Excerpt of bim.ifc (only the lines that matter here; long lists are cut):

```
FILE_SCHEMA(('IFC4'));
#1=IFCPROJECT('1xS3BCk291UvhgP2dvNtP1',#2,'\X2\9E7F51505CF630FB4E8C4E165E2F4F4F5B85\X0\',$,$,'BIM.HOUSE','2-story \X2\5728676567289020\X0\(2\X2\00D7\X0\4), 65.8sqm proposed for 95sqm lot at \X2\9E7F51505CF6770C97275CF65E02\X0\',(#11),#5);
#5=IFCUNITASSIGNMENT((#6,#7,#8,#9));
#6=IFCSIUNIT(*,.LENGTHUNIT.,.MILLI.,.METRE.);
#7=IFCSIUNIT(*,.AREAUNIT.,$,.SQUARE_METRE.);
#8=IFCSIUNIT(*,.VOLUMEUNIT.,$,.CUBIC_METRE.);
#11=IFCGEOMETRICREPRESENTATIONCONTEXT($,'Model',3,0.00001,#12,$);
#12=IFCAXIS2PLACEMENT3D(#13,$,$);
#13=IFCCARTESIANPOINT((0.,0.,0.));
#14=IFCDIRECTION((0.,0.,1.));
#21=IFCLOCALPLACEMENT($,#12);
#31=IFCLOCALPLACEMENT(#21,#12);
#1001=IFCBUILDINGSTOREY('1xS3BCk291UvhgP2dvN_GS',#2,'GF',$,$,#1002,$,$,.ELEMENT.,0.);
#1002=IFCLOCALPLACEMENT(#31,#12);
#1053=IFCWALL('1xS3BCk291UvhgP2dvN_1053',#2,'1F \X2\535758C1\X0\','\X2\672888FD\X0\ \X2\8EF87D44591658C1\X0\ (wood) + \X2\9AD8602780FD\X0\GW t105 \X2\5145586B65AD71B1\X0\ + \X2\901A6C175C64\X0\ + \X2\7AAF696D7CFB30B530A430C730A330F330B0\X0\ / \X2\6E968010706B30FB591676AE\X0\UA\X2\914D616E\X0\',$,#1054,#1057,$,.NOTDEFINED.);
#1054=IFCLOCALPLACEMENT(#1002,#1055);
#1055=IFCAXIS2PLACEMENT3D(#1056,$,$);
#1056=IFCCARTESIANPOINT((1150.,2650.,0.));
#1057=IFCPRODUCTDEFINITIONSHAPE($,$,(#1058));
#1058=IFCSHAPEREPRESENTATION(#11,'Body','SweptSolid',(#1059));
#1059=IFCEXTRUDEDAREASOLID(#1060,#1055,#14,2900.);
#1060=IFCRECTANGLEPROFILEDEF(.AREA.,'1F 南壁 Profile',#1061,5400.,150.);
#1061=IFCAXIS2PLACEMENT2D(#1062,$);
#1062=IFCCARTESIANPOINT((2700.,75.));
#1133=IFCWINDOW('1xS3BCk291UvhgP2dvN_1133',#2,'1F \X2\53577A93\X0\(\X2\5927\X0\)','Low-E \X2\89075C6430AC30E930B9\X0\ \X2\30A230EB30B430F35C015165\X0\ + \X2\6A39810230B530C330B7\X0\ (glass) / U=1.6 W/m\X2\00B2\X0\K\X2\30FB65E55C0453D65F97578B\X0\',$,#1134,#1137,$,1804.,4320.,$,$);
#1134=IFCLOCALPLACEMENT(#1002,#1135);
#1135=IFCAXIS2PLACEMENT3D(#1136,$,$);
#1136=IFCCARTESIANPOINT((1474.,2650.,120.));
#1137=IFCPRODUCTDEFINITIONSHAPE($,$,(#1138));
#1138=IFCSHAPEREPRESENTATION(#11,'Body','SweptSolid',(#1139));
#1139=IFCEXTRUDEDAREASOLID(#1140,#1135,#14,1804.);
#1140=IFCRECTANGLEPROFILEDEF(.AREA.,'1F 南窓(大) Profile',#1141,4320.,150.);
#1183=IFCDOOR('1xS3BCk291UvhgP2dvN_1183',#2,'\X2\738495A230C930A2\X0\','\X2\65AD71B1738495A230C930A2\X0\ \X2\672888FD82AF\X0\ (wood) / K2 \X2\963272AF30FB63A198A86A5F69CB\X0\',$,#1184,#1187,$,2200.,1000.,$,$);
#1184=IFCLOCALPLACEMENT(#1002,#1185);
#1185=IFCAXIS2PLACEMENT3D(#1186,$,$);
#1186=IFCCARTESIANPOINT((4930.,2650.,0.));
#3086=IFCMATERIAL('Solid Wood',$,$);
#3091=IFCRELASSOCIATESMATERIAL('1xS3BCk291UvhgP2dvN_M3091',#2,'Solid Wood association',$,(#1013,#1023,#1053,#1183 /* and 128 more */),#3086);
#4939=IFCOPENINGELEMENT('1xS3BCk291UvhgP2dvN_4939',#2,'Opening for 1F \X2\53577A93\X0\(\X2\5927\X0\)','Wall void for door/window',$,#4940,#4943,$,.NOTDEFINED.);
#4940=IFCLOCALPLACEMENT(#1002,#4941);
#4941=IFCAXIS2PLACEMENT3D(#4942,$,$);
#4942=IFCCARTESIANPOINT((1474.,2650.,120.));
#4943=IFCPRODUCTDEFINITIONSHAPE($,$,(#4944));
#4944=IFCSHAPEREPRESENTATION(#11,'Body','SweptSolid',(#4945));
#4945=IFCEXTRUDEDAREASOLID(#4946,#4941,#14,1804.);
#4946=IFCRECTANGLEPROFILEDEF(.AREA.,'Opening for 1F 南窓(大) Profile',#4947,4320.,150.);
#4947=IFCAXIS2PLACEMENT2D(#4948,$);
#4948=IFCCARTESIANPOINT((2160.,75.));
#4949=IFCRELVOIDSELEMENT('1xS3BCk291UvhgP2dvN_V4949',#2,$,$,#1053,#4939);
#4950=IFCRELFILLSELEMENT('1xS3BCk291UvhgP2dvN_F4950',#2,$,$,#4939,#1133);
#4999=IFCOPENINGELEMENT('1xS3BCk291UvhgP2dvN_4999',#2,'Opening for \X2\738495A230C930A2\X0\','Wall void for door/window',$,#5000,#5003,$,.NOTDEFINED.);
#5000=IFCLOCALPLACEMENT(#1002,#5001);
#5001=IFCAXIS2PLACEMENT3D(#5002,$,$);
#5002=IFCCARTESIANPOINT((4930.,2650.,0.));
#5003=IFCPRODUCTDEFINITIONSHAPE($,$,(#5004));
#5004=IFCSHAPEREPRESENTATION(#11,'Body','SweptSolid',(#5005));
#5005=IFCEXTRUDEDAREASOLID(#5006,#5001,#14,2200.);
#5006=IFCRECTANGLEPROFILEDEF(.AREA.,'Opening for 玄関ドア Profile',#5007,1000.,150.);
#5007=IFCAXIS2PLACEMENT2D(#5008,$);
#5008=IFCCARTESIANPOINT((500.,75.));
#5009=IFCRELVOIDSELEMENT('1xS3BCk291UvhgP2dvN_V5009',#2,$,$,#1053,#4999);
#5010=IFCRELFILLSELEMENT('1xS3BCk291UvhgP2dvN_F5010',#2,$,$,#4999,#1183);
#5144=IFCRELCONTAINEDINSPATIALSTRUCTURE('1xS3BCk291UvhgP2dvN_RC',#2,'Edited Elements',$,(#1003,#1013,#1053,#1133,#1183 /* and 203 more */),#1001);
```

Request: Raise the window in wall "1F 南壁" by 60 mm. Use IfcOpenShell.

```python
import numpy as np
import ifcopenshell
import ifcopenshell.api.geometry
import ifcopenshell.util.placement
import ifcopenshell.util.unit

model = ifcopenshell.open("bim.ifc")
unit_scale = ifcopenshell.util.unit.calculate_unit_scale(model)

window = model.by_guid("1xS3BCk291UvhgP2dvN_1133")
opening = window.FillsVoids[0].RelatingOpeningElement
dz = 60.0

shift = np.array([0.0, 0.0, dz])
# The window is not placed relative to its opening, so move both.
for product in (opening, window):
    matrix = ifcopenshell.util.placement.get_local_placement(product.ObjectPlacement)
    matrix[:3, 3] += shift
    ifcopenshell.api.geometry.edit_object_placement(model, product=product, matrix=matrix, is_si=False)

print(f"moved by {dz * unit_scale:+.3f} m")

model.write("bim-out.ifc")
```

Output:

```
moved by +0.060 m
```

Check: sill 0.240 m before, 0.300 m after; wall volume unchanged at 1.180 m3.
